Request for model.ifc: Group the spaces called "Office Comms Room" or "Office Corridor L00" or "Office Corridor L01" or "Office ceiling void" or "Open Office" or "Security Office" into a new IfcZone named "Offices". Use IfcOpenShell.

First a look at what the model holds.

```python
import ifcopenshell

model = ifcopenshell.open("model.ifc")
print(model.schema)
seen = {}
for space in model.by_type("IfcSpace"):
    seen[space.LongName] = seen.get(space.LongName, 0) + 1
for name, count in sorted(seen.items(), key=str):
    print(count, "x", name)
print("zones:", [z.Name for z in model.by_type("IfcZone")][:20])
```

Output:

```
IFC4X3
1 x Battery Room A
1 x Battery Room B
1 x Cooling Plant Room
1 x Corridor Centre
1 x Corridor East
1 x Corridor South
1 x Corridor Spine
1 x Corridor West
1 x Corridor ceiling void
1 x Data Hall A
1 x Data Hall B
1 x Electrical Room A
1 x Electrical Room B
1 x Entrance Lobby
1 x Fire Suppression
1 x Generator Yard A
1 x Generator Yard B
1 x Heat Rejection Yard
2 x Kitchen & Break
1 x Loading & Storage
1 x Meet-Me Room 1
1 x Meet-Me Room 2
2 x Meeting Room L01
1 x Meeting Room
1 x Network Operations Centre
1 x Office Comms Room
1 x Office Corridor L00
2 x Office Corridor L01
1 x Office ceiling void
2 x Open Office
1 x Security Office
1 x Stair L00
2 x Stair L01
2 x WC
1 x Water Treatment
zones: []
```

```python
import ifcopenshell
import ifcopenshell.api.group
import ifcopenshell.api.root

model = ifcopenshell.open("model.ifc")

names = {"Office Comms Room", "Office Corridor L00", "Office Corridor L01", "Office ceiling void", "Open Office", "Security Office"}
spaces = [s for s in model.by_type("IfcSpace") if s.LongName in names]

zone = ifcopenshell.api.root.create_entity(model, ifc_class="IfcZone", name="Offices")
ifcopenshell.api.group.assign_group(model, products=spaces, group=zone)
print(len(spaces), "spaces in", zone.Name)

model.write("model_edited.ifc")
```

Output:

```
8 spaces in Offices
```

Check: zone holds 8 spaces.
